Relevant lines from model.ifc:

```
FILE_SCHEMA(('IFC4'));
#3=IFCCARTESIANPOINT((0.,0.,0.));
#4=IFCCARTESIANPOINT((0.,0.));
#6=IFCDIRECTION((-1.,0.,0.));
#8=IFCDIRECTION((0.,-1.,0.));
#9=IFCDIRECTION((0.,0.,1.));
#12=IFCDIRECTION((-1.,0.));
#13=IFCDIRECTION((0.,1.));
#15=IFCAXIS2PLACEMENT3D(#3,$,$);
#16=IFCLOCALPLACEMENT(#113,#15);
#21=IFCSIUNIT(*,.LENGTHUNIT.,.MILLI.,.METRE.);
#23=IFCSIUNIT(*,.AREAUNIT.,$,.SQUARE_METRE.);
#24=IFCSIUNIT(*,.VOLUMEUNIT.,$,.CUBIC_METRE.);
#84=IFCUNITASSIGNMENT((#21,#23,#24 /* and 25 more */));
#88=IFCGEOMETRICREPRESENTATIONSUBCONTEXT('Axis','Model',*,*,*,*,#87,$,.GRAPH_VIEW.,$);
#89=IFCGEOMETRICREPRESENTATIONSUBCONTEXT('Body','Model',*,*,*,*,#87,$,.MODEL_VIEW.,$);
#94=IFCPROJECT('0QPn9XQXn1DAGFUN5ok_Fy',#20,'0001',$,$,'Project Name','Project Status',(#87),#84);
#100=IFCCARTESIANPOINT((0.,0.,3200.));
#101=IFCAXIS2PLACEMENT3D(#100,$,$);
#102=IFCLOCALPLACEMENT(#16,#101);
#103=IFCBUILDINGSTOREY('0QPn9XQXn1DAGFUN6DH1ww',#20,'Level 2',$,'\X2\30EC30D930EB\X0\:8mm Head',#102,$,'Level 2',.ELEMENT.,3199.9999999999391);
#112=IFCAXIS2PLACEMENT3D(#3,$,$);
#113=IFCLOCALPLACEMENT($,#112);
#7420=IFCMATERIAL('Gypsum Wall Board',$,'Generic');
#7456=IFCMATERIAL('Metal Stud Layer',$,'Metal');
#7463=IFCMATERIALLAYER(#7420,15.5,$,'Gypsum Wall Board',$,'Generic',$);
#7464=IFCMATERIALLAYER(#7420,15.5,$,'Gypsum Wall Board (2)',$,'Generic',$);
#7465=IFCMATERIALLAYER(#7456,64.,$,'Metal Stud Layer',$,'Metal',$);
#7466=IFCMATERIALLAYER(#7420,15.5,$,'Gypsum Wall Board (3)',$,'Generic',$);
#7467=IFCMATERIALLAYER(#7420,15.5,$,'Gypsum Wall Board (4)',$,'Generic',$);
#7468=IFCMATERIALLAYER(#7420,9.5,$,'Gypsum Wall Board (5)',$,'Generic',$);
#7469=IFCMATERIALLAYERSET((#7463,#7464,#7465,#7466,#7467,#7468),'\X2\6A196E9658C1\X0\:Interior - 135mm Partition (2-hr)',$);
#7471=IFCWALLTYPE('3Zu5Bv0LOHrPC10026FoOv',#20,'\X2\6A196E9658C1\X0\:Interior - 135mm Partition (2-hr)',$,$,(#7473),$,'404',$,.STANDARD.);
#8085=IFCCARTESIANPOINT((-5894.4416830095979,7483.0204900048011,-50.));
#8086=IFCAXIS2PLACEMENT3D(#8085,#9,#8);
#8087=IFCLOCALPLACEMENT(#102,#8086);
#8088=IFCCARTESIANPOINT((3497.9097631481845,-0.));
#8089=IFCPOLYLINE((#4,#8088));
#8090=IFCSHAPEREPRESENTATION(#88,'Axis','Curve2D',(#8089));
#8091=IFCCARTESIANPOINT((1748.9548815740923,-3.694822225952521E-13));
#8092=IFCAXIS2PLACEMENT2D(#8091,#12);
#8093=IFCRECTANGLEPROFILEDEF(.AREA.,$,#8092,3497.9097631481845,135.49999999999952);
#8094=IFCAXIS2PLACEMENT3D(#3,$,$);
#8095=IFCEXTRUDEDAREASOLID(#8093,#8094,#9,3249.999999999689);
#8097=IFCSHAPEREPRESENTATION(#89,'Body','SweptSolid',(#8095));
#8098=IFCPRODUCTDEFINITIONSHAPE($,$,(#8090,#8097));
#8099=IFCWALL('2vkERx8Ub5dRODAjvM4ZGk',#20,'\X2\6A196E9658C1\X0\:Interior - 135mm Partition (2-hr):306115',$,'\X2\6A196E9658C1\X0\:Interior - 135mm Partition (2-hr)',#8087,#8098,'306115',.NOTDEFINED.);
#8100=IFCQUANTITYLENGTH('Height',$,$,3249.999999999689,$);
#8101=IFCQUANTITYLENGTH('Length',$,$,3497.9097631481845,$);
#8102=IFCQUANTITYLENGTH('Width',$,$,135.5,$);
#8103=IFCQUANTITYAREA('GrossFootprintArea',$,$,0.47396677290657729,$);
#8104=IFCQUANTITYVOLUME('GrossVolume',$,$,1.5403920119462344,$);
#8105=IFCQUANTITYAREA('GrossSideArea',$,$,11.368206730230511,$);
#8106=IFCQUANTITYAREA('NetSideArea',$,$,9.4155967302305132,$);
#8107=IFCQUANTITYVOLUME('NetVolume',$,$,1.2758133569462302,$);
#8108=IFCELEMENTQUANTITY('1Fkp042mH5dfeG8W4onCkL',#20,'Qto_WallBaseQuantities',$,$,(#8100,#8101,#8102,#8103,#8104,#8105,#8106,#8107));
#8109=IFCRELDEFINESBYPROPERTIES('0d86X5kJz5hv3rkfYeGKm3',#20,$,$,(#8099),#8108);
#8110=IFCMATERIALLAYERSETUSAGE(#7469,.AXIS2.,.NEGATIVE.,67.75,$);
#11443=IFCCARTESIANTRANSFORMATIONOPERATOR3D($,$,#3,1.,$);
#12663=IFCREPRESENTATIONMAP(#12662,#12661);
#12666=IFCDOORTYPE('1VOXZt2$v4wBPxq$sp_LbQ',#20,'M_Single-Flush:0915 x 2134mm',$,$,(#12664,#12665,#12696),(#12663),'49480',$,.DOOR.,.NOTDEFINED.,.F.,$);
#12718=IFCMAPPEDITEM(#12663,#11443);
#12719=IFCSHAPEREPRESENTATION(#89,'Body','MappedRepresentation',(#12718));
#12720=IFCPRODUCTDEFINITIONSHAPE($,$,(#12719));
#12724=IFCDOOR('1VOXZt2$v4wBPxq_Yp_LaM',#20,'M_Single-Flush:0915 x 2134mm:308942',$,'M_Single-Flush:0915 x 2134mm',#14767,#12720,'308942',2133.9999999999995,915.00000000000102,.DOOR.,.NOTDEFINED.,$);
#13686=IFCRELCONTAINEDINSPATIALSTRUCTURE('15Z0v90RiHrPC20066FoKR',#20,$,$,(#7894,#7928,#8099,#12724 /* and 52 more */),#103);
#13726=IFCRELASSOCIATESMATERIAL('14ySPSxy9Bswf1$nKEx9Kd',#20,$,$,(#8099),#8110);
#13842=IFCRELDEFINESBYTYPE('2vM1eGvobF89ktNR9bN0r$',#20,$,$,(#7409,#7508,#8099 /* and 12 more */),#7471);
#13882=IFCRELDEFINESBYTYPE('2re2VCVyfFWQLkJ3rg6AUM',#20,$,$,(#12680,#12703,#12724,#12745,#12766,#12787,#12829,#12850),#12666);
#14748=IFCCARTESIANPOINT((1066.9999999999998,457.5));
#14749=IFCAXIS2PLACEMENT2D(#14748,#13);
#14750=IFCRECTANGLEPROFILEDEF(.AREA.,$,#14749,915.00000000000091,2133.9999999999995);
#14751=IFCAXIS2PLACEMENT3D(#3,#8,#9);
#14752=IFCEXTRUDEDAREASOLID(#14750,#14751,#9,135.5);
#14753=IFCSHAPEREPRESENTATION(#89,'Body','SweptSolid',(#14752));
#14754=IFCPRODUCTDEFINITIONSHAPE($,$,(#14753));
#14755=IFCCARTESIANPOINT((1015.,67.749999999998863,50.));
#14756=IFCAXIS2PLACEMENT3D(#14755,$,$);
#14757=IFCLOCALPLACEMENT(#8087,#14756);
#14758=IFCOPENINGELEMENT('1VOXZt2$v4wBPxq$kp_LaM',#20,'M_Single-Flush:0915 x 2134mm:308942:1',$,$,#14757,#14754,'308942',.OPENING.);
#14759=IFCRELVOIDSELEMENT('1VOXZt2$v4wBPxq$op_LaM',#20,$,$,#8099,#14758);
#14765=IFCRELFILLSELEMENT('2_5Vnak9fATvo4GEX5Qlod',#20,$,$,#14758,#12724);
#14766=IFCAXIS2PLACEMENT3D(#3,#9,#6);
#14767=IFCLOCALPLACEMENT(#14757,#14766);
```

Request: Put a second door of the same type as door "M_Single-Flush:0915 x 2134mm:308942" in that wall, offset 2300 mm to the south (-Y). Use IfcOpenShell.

```python
import ifcopenshell
import ifcopenshell.api.feature
import ifcopenshell.api.geometry
import ifcopenshell.api.pset
import ifcopenshell.api.root
import ifcopenshell.geom
import ifcopenshell.util.element
import ifcopenshell.util.placement
import ifcopenshell.util.shape
import ifcopenshell.util.unit

model = ifcopenshell.open("model.ifc")
unit_scale = ifcopenshell.util.unit.calculate_unit_scale(model)
area_scale = ifcopenshell.util.unit.calculate_unit_scale(model, "AREAUNIT")
volume_scale = ifcopenshell.util.unit.calculate_unit_scale(model, "VOLUMEUNIT")
settings = ifcopenshell.geom.settings()


def volume(element):
    """Net volume in cubic metres, openings subtracted."""
    shape = ifcopenshell.geom.create_shape(settings, element)
    return ifcopenshell.util.shape.get_volume(shape.geometry)


def reuse_history(source, copy):
    """copy_class also copies each property set's owner history, people and application; keep the originals."""
    for rel in copy.IsDefinedBy:
        if rel.is_a("IfcRelDefinesByProperties") and (history := rel.RelatingPropertyDefinition.OwnerHistory):
            rel.RelatingPropertyDefinition.OwnerHistory = source.OwnerHistory
            ifcopenshell.util.element.remove_deep2(model, history)


door = model.by_guid("1VOXZt2$v4wBPxq_Yp_LaM")
opening = door.FillsVoids[0].RelatingOpeningElement
wall = opening.VoidsElements[0].RelatingBuildingElement
before = volume(wall)
shift = ifcopenshell.util.placement.get_local_placement(wall.ObjectPlacement)[:3, 0] * 2.3 / unit_scale

# copy_class copies the void relationship, type, container and properties, but no geometry.
new_opening = ifcopenshell.api.root.copy_class(model, product=opening)
new_opening.Representation = ifcopenshell.util.element.copy_deep(
    model, opening.Representation, exclude=["IfcGeometricRepresentationContext", "IfcRepresentationMap"]
)
new_opening.Name = "M_Single-Flush:0915 x 2134mm"
new_opening.Tag = None
reuse_history(opening, new_opening)
new_door = ifcopenshell.api.root.copy_class(model, product=door)
new_door.Representation = ifcopenshell.util.element.copy_deep(
    model, door.Representation, exclude=["IfcGeometricRepresentationContext", "IfcRepresentationMap"]
)
new_door.Name = "M_Single-Flush:0915 x 2134mm"
new_door.Tag = None
reuse_history(door, new_door)
ifcopenshell.api.feature.add_filling(model, opening=new_opening, element=new_door)

for old, new in ((opening, new_opening), (door, new_door)):
    matrix = ifcopenshell.util.placement.get_local_placement(old.ObjectPlacement)
    matrix[:3, 3] += shift
    ifcopenshell.api.geometry.edit_object_placement(model, product=new, matrix=matrix, is_si=False)

after = volume(wall)
thickness = 0.1355  # wall thickness in metres

# Update the wall's stored quantities.
qto = model.by_id(ifcopenshell.util.element.get_pset(wall, "Qto_WallBaseQuantities", should_inherit=False)["id"])
ifcopenshell.api.pset.edit_qto(model, qto=qto, properties={
    "NetSideArea": after / thickness / area_scale,
    "NetVolume": after / volume_scale,
})

print(f"wall volume {before:.3f} -> {after:.3f} m3")

model.write("model_edited.ifc")
```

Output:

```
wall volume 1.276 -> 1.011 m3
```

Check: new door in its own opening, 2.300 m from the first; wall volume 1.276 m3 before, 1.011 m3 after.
